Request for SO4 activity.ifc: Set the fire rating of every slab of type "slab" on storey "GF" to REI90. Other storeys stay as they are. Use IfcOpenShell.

First a look at what the model holds.

```python
import ifcopenshell
import ifcopenshell.util.element

model = ifcopenshell.open("SO4 activity.ifc")
print(model.schema)
storey = next(s for s in model.by_type("IfcBuildingStorey") if s.Name == "GF")
slabs = [e for e in ifcopenshell.util.element.get_decomposition(storey) if e.is_a("IfcSlab")]
seen = {}
for e in slabs:
    element_type = ifcopenshell.util.element.get_type(e)
    key = (element_type.Name if element_type != e and element_type else None, ifcopenshell.util.element.get_pset(e, "Pset_SlabCommon", "FireRating"))
    seen[key] = seen.get(key, 0) + 1
for (name, value), count in sorted(seen.items(), key=str):
    print(count, "x", name, "|", value)
```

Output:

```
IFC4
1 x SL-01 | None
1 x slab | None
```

```python
import ifcopenshell
import ifcopenshell.api.pset
import ifcopenshell.util.element

model = ifcopenshell.open("SO4 activity.ifc")

storey = next(s for s in model.by_type("IfcBuildingStorey") if s.Name == "GF")
slabs = [e for e in ifcopenshell.util.element.get_decomposition(storey) if e.is_a("IfcSlab")]

count = 0
for e in slabs:
    element_type = ifcopenshell.util.element.get_type(e)
    if element_type in (None, e) or element_type.Name != "slab":
        continue
    # add_pset returns the element's existing set when there is one.
    pset = ifcopenshell.api.pset.add_pset(model, product=e, name="Pset_SlabCommon")
    ifcopenshell.api.pset.edit_pset(model, pset=pset, properties={"FireRating": "REI90"})
    count += 1

print(count, "slabs updated")

model.write("SO4 activity_v2.ifc")
```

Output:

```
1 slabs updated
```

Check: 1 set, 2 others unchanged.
